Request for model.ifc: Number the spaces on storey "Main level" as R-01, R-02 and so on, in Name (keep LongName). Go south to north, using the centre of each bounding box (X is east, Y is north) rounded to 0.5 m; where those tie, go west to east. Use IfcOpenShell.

First a look at what the model holds.

```python
import ifcopenshell
import ifcopenshell.util.element
import ifcopenshell.util.placement

model = ifcopenshell.open("model.ifc")
print(model.schema)
storey = next(s for s in model.by_type("IfcBuildingStorey") if s.Name == "Main level")
spaces = [e for e in ifcopenshell.util.element.get_decomposition(storey) if e.is_a("IfcSpace")]
for e in sorted(spaces, key=lambda e: e.id()):
    origin = ifcopenshell.util.placement.get_local_placement(e.ObjectPlacement)[:3, 3]
    print(e.id(), e.Name, e.LongName, origin.round(2) + 0.0, sep=" | ")
```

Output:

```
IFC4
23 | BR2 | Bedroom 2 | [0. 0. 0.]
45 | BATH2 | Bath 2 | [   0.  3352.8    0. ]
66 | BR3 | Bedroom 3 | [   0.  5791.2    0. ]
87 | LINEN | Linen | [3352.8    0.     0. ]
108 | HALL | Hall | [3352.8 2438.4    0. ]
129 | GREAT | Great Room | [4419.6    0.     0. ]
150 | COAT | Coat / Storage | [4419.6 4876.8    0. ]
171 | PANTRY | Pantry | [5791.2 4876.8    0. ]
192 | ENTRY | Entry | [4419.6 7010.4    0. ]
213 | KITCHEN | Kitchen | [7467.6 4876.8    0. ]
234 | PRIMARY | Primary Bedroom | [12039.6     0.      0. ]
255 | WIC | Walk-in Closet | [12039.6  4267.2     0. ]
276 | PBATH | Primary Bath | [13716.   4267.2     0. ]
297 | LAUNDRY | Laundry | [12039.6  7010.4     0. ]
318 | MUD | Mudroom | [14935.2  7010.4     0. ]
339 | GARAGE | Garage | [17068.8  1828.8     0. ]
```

```python
import ifcopenshell
import ifcopenshell.geom
import ifcopenshell.util.element
import ifcopenshell.util.shape

model = ifcopenshell.open("model.ifc")
settings = ifcopenshell.geom.settings()
settings.set("use-world-coords", True)


def centre(element):
    shape = ifcopenshell.geom.create_shape(settings, element)
    return ifcopenshell.util.shape.get_bbox_centroid(shape.geometry)


storey = next(s for s in model.by_type("IfcBuildingStorey") if s.Name == "Main level")
spaces = [e for e in ifcopenshell.util.element.get_decomposition(storey) if e.is_a("IfcSpace")]

# Insertion points can sit at a corner or the storey origin, so sort by the geometry (in metres).
centres = {e: centre(e) for e in spaces}
spaces.sort(key=lambda e: (round(centres[e][1] / 0.5), centres[e][0]))

for i, e in enumerate(spaces, start=1):
    number = f"R-{i:02d}"
    e.Name = number
    print(e.id(), number)

model.write("model_updated.ifc")
```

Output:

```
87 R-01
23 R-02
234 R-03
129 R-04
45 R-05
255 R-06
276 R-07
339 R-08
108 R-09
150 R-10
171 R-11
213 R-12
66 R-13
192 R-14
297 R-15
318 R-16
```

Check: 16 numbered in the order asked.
